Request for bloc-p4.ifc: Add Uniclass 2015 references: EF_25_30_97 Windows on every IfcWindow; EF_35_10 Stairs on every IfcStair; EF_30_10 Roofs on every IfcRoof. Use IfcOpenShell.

First a look at what the model holds.

```python
import ifcopenshell

model = ifcopenshell.open("bloc-p4.ifc")
print(model.schema)
print("classifications:", [c.Name for c in model.by_type("IfcClassification")])
for ifc_class in ("IfcDoor", "IfcRoof", "IfcStair", "IfcWall", "IfcWindow"):
    print(ifc_class, len(model.by_type(ifc_class)))
```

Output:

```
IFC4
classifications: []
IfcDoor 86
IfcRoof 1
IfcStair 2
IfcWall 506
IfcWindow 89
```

```python
import ifcopenshell
import ifcopenshell.api.classification

model = ifcopenshell.open("bloc-p4.ifc")

system = ifcopenshell.api.classification.add_classification(model, classification="Uniclass 2015")

codes = {
    "IfcWindow": ("EF_25_30_97", "Windows"),
    "IfcStair": ("EF_35_10", "Stairs"),
    "IfcRoof": ("EF_30_10", "Roofs"),
}
for ifc_class, (code, name) in codes.items():
    products = model.by_type(ifc_class)
    ifcopenshell.api.classification.add_reference(
        model, products=products, classification=system, identification=code, name=name
    )
    print(code, len(products))

model.write("bloc-p4_rev.ifc")
```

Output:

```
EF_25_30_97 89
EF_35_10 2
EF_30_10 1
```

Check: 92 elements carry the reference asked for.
